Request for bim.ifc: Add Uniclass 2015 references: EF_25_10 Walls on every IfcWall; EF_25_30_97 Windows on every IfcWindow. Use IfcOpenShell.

First a look at what the model holds.

```python
import ifcopenshell

model = ifcopenshell.open("bim.ifc")
print(model.schema)
print("classifications:", [c.Name for c in model.by_type("IfcClassification")])
for ifc_class in ("IfcDoor", "IfcRoof", "IfcStair", "IfcWall", "IfcWindow"):
    print(ifc_class, len(model.by_type(ifc_class)))
```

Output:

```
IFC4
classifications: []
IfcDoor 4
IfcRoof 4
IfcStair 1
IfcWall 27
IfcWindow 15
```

```python
import ifcopenshell
import ifcopenshell.api.classification

model = ifcopenshell.open("bim.ifc")

system = ifcopenshell.api.classification.add_classification(model, classification="Uniclass 2015")

codes = {
    "IfcWall": ("EF_25_10", "Walls"),
    "IfcWindow": ("EF_25_30_97", "Windows"),
}
for ifc_class, (code, name) in codes.items():
    products = model.by_type(ifc_class)
    ifcopenshell.api.classification.add_reference(
        model, products=products, classification=system, identification=code, name=name
    )
    print(code, len(products))

model.write("bim-out.ifc")
```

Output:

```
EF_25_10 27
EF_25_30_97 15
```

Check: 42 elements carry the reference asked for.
